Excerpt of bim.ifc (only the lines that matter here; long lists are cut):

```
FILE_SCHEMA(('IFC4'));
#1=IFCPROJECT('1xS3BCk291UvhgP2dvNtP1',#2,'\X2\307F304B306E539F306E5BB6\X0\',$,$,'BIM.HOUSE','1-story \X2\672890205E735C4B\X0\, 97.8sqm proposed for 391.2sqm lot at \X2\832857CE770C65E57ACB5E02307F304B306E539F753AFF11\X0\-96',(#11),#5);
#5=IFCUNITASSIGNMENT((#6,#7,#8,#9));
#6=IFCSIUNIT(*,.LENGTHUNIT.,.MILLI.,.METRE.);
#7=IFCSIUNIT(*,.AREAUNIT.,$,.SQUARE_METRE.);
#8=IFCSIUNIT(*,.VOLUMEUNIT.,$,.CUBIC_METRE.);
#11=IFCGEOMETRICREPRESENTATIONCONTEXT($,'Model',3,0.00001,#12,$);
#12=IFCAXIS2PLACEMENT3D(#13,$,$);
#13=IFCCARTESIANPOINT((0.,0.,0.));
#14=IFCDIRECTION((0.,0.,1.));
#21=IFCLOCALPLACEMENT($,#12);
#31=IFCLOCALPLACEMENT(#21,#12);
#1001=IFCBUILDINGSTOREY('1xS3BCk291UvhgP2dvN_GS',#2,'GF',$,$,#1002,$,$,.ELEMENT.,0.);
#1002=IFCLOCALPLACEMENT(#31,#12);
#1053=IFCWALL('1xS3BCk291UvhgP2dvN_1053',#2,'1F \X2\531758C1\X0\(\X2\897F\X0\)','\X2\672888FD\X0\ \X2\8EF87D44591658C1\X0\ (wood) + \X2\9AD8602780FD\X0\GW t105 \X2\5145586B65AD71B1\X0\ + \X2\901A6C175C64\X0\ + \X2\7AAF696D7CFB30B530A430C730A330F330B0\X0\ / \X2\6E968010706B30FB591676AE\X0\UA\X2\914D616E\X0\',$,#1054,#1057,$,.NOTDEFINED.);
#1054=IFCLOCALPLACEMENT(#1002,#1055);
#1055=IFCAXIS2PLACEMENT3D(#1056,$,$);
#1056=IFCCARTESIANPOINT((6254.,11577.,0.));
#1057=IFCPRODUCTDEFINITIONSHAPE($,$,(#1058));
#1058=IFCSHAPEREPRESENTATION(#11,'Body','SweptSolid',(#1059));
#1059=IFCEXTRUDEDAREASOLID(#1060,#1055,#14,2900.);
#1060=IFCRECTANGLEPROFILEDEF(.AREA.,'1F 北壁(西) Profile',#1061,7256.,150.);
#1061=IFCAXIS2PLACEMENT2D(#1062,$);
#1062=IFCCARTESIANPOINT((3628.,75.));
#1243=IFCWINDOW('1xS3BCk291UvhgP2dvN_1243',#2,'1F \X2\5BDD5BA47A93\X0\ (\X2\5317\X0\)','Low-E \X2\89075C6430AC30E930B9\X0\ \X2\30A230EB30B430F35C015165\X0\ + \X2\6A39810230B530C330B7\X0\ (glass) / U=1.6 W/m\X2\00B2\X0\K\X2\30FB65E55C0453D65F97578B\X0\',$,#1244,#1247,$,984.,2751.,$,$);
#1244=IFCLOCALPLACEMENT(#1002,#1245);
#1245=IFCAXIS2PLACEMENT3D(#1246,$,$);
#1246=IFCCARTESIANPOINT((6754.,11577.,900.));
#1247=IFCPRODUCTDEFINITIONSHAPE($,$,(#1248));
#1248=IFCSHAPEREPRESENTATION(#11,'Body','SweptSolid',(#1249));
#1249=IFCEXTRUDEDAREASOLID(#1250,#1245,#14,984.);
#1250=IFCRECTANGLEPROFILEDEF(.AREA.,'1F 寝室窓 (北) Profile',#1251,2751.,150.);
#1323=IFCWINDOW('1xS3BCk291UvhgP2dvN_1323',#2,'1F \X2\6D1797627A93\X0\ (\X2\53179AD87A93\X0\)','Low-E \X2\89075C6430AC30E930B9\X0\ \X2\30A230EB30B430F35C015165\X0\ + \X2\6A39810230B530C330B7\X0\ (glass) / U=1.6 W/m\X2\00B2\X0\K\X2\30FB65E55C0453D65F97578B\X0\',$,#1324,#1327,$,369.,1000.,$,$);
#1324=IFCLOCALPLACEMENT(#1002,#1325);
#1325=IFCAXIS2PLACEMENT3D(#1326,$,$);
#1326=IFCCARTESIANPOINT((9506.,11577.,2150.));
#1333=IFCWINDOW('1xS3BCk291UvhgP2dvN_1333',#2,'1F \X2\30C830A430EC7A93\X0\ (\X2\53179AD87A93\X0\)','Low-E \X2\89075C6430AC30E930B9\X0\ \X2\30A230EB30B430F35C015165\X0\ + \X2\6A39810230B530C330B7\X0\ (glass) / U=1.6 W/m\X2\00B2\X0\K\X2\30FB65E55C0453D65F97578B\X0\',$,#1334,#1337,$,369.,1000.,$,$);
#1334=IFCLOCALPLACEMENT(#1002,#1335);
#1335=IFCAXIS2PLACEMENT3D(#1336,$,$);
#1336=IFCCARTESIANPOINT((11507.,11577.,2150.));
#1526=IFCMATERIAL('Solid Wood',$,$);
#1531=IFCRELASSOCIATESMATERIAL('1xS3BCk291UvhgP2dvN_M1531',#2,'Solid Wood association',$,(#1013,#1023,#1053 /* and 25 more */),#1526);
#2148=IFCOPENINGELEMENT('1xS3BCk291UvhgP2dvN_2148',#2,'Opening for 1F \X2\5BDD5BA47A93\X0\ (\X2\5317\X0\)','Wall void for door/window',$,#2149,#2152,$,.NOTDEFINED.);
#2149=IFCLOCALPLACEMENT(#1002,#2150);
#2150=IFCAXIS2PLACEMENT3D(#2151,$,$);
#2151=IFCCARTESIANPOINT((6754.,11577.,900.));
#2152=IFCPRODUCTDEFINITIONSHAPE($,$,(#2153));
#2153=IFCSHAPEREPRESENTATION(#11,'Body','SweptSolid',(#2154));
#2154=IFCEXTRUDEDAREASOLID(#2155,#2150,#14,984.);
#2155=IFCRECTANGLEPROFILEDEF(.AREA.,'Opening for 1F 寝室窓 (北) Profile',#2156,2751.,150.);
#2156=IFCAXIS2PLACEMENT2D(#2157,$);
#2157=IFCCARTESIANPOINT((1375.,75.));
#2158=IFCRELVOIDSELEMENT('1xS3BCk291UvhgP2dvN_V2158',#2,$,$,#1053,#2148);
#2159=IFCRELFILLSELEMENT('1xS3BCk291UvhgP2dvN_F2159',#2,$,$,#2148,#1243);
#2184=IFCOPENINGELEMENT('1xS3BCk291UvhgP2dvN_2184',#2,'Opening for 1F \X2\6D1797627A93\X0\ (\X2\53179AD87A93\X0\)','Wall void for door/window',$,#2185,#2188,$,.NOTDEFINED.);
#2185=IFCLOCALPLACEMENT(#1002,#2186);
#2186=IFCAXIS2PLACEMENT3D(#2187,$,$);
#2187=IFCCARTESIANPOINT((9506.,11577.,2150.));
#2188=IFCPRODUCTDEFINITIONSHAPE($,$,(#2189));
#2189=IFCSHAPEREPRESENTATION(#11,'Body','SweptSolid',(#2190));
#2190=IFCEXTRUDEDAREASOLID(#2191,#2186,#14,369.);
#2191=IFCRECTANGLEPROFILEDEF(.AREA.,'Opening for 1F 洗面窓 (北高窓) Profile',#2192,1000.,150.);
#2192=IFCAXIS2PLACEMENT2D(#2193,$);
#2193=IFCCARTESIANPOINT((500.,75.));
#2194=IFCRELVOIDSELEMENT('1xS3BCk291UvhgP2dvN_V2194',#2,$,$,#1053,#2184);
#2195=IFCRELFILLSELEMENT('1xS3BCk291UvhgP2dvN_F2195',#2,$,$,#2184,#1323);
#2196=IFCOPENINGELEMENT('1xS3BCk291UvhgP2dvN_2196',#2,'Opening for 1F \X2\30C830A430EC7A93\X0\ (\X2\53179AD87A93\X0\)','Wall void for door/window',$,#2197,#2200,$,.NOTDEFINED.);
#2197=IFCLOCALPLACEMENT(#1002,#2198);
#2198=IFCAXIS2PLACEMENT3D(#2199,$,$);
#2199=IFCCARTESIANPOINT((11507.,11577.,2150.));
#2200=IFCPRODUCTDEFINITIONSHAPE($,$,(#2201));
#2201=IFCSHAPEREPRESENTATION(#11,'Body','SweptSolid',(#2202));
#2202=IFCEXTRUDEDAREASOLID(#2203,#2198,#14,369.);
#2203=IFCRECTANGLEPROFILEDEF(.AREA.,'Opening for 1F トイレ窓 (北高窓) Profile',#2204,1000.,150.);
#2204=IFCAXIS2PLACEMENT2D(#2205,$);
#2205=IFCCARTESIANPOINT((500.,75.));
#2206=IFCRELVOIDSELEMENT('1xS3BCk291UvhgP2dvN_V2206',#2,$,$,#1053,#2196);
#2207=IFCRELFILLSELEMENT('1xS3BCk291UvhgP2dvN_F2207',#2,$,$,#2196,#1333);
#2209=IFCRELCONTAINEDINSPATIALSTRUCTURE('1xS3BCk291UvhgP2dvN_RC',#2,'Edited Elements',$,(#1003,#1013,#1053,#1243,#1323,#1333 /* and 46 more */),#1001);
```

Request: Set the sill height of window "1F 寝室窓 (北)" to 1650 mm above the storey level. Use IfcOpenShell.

```python
import numpy as np
import ifcopenshell
import ifcopenshell.api.geometry
import ifcopenshell.geom
import ifcopenshell.util.element
import ifcopenshell.util.placement
import ifcopenshell.util.shape
import ifcopenshell.util.unit

model = ifcopenshell.open("bim.ifc")
unit_scale = ifcopenshell.util.unit.calculate_unit_scale(model)

window = model.by_guid("1xS3BCk291UvhgP2dvN_1243")
opening = window.FillsVoids[0].RelatingOpeningElement
storey = ifcopenshell.util.element.get_container(window, ifc_class="IfcBuildingStorey")
level = ifcopenshell.util.placement.get_local_placement(storey.ObjectPlacement)[2, 3]

# The opening's origin need not be at the sill, so measure its lowest point.
shape = ifcopenshell.geom.create_shape(ifcopenshell.geom.settings(), opening)
bottom = ifcopenshell.util.shape.get_shape_bottom_elevation(shape, shape.geometry) / unit_scale
dz = level + 1650.0 - bottom

shift = np.array([0.0, 0.0, dz])
# The window is not placed relative to its opening, so move both.
for product in (opening, window):
    matrix = ifcopenshell.util.placement.get_local_placement(product.ObjectPlacement)
    matrix[:3, 3] += shift
    ifcopenshell.api.geometry.edit_object_placement(model, product=product, matrix=matrix, is_si=False)

print(f"moved by {dz * unit_scale:+.3f} m")

model.write("bim-out.ifc")
```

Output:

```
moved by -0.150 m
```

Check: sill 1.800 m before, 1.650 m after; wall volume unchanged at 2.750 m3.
